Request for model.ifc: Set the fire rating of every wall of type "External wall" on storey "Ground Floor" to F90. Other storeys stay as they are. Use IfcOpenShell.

First a look at what the model holds.

```python
import ifcopenshell
import ifcopenshell.util.element

model = ifcopenshell.open("model.ifc")
print(model.schema)
storey = next(s for s in model.by_type("IfcBuildingStorey") if s.Name == "Ground Floor")
walls = [e for e in ifcopenshell.util.element.get_decomposition(storey) if e.is_a("IfcWall")]
seen = {}
for e in walls:
    element_type = ifcopenshell.util.element.get_type(e)
    key = (element_type.Name if element_type != e and element_type else None, ifcopenshell.util.element.get_pset(e, "Pset_WallCommon", "FireRating"))
    seen[key] = seen.get(key, 0) + 1
for (name, value), count in sorted(seen.items(), key=str):
    print(count, "x", name, "|", value)
```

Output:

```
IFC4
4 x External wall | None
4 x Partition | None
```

```python
import ifcopenshell
import ifcopenshell.api.pset
import ifcopenshell.util.element

model = ifcopenshell.open("model.ifc")

storey = next(s for s in model.by_type("IfcBuildingStorey") if s.Name == "Ground Floor")
walls = [e for e in ifcopenshell.util.element.get_decomposition(storey) if e.is_a("IfcWall")]

count = 0
for e in walls:
    element_type = ifcopenshell.util.element.get_type(e)
    if element_type in (None, e) or element_type.Name != "External wall":
        continue
    # add_pset returns the element's existing set when there is one.
    pset = ifcopenshell.api.pset.add_pset(model, product=e, name="Pset_WallCommon")
    ifcopenshell.api.pset.edit_pset(model, pset=pset, properties={"FireRating": "F90"})
    count += 1

print(count, "walls updated")

model.write("model_updated.ifc")
```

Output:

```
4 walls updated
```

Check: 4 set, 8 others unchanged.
